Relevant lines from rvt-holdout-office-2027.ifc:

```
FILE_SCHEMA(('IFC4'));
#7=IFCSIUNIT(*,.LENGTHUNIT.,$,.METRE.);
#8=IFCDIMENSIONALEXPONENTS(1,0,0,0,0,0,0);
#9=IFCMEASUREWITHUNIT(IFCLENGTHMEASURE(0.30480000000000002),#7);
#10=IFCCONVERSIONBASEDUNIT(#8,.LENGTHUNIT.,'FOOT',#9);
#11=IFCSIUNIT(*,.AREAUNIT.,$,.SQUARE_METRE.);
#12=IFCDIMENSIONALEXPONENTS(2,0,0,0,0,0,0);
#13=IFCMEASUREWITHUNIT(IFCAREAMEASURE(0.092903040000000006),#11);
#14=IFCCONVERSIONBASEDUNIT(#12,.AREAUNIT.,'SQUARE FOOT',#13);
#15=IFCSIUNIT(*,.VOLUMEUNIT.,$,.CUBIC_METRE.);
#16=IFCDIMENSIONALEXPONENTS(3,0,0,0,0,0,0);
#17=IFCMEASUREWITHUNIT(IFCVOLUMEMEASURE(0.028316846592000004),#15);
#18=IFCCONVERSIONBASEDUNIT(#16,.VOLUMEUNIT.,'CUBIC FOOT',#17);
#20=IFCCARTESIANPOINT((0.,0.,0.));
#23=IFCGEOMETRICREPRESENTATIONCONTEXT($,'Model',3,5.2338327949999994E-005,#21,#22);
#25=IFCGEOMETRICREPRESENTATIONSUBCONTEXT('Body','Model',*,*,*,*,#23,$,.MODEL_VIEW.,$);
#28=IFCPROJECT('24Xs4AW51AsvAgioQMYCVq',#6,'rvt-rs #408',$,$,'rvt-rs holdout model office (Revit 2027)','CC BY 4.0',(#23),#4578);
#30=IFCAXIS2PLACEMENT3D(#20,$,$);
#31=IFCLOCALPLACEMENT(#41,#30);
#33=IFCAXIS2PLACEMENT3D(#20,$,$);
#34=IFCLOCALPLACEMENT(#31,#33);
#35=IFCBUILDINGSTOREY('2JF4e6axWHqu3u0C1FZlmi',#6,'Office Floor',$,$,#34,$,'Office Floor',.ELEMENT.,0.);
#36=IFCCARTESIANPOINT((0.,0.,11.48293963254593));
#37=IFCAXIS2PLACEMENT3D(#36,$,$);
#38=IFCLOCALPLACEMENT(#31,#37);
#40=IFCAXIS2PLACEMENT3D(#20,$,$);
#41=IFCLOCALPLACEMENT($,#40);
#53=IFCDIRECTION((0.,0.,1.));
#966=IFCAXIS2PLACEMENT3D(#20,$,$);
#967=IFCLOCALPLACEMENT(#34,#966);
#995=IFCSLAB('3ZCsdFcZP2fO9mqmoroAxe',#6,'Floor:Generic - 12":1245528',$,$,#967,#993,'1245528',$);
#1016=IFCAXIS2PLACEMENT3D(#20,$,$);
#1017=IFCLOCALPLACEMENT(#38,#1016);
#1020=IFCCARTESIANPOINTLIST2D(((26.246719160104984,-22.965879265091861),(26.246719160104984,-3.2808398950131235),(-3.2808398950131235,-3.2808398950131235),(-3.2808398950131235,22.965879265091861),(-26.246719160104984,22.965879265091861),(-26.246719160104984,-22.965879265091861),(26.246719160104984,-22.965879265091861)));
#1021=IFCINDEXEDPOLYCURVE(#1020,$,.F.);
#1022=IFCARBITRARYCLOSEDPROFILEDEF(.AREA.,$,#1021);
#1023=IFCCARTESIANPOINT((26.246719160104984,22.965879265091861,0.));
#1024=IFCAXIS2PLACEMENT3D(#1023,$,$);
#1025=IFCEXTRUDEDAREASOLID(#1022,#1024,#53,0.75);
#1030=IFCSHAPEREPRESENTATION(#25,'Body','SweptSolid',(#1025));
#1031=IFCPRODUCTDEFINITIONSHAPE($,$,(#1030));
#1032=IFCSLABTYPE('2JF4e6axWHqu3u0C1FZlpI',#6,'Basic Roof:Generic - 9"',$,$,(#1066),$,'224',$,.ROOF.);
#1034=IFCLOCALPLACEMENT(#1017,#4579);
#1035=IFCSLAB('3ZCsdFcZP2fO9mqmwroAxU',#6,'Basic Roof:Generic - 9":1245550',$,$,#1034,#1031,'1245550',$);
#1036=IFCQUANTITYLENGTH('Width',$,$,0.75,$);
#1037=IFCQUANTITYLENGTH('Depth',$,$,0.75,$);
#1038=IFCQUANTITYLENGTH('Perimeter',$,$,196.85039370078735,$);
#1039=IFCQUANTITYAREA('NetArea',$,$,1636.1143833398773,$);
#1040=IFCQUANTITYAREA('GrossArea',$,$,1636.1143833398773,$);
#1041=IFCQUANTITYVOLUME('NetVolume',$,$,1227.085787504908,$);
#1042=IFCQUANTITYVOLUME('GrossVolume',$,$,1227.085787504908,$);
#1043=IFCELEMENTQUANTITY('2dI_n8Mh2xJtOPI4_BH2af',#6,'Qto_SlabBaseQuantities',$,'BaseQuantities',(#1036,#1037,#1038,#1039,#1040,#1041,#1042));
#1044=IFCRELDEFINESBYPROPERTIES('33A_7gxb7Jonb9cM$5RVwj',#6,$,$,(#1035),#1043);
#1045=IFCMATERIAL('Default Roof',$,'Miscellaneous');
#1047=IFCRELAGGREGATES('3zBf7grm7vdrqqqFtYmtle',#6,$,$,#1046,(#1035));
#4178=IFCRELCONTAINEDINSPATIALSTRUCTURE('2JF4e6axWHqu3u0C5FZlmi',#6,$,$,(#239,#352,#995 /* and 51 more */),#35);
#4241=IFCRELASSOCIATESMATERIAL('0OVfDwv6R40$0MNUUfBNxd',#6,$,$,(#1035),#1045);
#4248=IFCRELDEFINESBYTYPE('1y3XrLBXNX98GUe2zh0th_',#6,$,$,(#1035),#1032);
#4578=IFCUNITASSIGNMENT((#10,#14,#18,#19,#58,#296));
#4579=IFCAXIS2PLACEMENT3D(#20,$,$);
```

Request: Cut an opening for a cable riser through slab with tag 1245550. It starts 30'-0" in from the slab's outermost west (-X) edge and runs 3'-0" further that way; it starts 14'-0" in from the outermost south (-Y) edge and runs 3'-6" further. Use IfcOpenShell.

```python
import numpy as np
import ifcopenshell
import ifcopenshell.api.feature
import ifcopenshell.api.geometry
import ifcopenshell.api.pset
import ifcopenshell.api.root
import ifcopenshell.geom
import ifcopenshell.util.element
import ifcopenshell.util.placement
import ifcopenshell.util.representation
import ifcopenshell.util.shape
import ifcopenshell.util.unit

model = ifcopenshell.open("rvt-holdout-office-2027.ifc")
unit_scale = ifcopenshell.util.unit.calculate_unit_scale(model)
area_scale = ifcopenshell.util.unit.calculate_unit_scale(model, "AREAUNIT")
volume_scale = ifcopenshell.util.unit.calculate_unit_scale(model, "VOLUMEUNIT")
settings = ifcopenshell.geom.settings()


def volume(element):
    """Net volume in cubic metres, openings subtracted."""
    shape = ifcopenshell.geom.create_shape(settings, element)
    return ifcopenshell.util.shape.get_volume(shape.geometry)


slab = model.by_id(1035)
before = volume(slab)

# Extent in the slab's own axes, in metres. The edges named are its -X and -Y sides.
slab_shape = ifcopenshell.geom.create_shape(settings, slab)
vertices = ifcopenshell.util.shape.get_vertices(slab_shape.geometry)
x_min, y_min, bottom = vertices.min(axis=0)
top = vertices[:, 2].max()

opening = ifcopenshell.api.root.create_entity(model, ifc_class="IfcOpeningElement", name="Cable riser opening", predefined_type="OPENING")
context = ifcopenshell.util.representation.get_context(model, "Model", "Body", "MODEL_VIEW")
width, depth = 0.9144, 1.0668
outline = [(0.0, 0.0), (width, 0.0), (width, depth), (0.0, depth), (0.0, 0.0)]
# Overshoot both faces by 50 mm so the cut is clean.
shape = ifcopenshell.api.geometry.add_slab_representation(
    model, context=context, depth=top - bottom + 0.1, polyline=outline
)
ifcopenshell.api.geometry.assign_representation(model, product=opening, representation=shape)

matrix = ifcopenshell.util.placement.get_local_placement(slab.ObjectPlacement)
matrix[:, 3] = matrix @ np.append(np.array([x_min + 9.144, y_min + 4.2672, bottom - 0.05]) / unit_scale, 1.0)
ifcopenshell.api.geometry.edit_object_placement(model, product=opening, matrix=matrix, is_si=False)
ifcopenshell.api.feature.add_feature(model, feature=opening, element=slab)

after = volume(slab)

# Update the slab's stored quantities.
qto = model.by_id(ifcopenshell.util.element.get_pset(slab, "Qto_SlabBaseQuantities", should_inherit=False)["id"])
ifcopenshell.api.pset.edit_qto(model, qto=qto, properties={
    "NetArea": after / (top - bottom) / area_scale,
    "NetVolume": after / volume_scale,
})

print(f"slab volume {before:.3f} -> {after:.3f} m3")

model.write("rvt-holdout-office-2027_rev.ifc")
```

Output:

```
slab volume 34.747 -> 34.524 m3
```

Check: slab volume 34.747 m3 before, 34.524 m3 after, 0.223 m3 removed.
